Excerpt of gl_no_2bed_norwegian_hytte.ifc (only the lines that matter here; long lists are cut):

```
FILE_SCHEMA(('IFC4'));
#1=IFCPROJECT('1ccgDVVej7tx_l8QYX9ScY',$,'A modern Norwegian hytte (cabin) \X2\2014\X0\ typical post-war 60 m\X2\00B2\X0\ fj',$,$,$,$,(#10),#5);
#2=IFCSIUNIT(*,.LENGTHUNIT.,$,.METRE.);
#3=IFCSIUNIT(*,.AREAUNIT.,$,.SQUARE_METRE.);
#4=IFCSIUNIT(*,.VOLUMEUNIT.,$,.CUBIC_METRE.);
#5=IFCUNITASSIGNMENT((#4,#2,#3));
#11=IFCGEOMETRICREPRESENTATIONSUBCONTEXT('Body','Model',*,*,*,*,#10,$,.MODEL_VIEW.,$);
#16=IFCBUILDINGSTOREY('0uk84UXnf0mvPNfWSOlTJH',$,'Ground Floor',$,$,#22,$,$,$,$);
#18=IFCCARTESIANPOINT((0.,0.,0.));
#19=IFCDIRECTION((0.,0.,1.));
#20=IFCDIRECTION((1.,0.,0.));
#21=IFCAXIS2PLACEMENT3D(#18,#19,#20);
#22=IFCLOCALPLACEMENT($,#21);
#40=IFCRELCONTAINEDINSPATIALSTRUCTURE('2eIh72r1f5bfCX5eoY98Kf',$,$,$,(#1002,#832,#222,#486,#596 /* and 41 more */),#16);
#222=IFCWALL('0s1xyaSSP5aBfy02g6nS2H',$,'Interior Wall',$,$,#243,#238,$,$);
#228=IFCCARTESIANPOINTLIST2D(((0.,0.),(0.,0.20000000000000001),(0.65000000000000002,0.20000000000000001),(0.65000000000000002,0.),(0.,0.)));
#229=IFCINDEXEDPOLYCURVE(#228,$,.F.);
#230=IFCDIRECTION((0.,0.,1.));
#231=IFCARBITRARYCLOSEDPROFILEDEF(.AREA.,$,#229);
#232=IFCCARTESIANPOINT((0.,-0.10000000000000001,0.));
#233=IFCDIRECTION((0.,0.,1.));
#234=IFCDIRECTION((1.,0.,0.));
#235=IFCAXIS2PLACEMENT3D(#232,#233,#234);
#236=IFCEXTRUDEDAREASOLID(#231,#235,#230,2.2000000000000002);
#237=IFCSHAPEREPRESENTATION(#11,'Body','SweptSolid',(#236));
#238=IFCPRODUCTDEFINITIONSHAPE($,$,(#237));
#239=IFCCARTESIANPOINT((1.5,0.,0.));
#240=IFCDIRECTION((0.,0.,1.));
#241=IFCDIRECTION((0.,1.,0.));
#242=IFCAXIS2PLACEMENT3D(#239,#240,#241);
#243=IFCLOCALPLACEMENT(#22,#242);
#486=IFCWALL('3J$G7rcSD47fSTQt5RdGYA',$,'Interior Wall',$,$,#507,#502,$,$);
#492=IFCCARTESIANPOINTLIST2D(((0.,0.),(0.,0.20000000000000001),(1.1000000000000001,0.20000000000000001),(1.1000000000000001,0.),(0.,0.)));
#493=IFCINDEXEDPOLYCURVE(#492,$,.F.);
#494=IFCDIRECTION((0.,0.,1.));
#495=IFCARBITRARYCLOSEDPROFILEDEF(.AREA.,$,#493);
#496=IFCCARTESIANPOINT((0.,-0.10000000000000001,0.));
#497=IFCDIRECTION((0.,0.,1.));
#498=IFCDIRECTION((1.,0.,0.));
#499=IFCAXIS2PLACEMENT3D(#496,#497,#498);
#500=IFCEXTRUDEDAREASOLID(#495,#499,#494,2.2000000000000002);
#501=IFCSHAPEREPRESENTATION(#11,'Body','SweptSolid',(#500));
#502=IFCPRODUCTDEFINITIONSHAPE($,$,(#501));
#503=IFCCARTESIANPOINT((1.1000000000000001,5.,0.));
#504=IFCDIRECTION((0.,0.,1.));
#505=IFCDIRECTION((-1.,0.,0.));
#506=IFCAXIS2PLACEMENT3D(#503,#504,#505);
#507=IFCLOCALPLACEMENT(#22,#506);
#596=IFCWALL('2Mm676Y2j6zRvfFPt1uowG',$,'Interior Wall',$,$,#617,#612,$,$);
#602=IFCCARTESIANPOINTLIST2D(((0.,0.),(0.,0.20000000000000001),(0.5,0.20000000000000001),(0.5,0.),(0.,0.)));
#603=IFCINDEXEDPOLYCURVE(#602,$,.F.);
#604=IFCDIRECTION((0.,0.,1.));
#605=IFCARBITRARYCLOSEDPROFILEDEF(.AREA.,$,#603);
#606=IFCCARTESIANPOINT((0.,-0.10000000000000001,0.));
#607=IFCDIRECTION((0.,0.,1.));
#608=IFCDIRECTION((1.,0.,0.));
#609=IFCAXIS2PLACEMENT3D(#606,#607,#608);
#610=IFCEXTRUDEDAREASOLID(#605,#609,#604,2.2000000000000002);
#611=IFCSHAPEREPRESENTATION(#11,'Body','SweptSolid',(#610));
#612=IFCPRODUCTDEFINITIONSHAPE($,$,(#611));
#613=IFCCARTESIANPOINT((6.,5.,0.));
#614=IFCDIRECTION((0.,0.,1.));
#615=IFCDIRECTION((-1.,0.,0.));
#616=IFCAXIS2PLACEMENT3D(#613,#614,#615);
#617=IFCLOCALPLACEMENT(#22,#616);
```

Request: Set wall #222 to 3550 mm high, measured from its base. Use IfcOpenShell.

```python
import ifcopenshell
import ifcopenshell.geom
import ifcopenshell.util.representation
import ifcopenshell.util.shape

model = ifcopenshell.open("gl_no_2bed_norwegian_hytte.ifc")
settings = ifcopenshell.geom.settings()


def volume(element):
    """Net volume in cubic metres, openings subtracted."""
    shape = ifcopenshell.geom.create_shape(settings, element)
    return ifcopenshell.util.shape.get_volume(shape.geometry)


wall = model.by_guid("0s1xyaSSP5aBfy02g6nS2H")
before = volume(wall)

body = ifcopenshell.util.representation.get_representation(wall, "Model", "Body")
solid = body.Items[0]
old_height = solid.Depth
solid.Depth = 3.55
after = volume(wall)

print(f"height {old_height:g} -> {solid.Depth:g}, volume {before:.3f} -> {after:.3f} m3")

model.write("gl_no_2bed_norwegian_hytte_edited.ifc")
```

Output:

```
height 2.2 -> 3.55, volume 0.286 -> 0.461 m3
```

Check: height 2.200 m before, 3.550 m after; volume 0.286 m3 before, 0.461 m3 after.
